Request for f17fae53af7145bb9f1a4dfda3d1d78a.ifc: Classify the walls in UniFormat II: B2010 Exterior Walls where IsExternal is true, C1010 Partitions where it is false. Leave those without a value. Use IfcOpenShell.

First a look at what the model holds.

```python
import ifcopenshell
import ifcopenshell.util.element

model = ifcopenshell.open("f17fae53af7145bb9f1a4dfda3d1d78a.ifc")
print(model.schema)
print("classifications:", [c.Name for c in model.by_type("IfcClassification")])
values = [ifcopenshell.util.element.get_pset(e, "Pset_WallCommon", "IsExternal") for e in model.by_type("IfcWall")]
for value in (True, False, None):
    print("IsExternal", value, values.count(value))
```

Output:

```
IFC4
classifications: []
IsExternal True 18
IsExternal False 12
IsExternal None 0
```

```python
import ifcopenshell
import ifcopenshell.api.classification
import ifcopenshell.util.element

model = ifcopenshell.open("f17fae53af7145bb9f1a4dfda3d1d78a.ifc")

system = ifcopenshell.api.classification.add_classification(model, classification="UniFormat II")

walls = model.by_type("IfcWall")
external = {e: ifcopenshell.util.element.get_pset(e, "Pset_WallCommon", "IsExternal") for e in walls}
for flag, code, name in ((True, "B2010", "Exterior Walls"), (False, "C1010", "Partitions")):
    products = [e for e in walls if external[e] is flag]
    ifcopenshell.api.classification.add_reference(
        model, products=products, classification=system, identification=code, name=name
    )
    print(code, len(products))

model.write("f17fae53af7145bb9f1a4dfda3d1d78a_edited.ifc")
```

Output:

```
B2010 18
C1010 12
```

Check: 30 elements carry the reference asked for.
